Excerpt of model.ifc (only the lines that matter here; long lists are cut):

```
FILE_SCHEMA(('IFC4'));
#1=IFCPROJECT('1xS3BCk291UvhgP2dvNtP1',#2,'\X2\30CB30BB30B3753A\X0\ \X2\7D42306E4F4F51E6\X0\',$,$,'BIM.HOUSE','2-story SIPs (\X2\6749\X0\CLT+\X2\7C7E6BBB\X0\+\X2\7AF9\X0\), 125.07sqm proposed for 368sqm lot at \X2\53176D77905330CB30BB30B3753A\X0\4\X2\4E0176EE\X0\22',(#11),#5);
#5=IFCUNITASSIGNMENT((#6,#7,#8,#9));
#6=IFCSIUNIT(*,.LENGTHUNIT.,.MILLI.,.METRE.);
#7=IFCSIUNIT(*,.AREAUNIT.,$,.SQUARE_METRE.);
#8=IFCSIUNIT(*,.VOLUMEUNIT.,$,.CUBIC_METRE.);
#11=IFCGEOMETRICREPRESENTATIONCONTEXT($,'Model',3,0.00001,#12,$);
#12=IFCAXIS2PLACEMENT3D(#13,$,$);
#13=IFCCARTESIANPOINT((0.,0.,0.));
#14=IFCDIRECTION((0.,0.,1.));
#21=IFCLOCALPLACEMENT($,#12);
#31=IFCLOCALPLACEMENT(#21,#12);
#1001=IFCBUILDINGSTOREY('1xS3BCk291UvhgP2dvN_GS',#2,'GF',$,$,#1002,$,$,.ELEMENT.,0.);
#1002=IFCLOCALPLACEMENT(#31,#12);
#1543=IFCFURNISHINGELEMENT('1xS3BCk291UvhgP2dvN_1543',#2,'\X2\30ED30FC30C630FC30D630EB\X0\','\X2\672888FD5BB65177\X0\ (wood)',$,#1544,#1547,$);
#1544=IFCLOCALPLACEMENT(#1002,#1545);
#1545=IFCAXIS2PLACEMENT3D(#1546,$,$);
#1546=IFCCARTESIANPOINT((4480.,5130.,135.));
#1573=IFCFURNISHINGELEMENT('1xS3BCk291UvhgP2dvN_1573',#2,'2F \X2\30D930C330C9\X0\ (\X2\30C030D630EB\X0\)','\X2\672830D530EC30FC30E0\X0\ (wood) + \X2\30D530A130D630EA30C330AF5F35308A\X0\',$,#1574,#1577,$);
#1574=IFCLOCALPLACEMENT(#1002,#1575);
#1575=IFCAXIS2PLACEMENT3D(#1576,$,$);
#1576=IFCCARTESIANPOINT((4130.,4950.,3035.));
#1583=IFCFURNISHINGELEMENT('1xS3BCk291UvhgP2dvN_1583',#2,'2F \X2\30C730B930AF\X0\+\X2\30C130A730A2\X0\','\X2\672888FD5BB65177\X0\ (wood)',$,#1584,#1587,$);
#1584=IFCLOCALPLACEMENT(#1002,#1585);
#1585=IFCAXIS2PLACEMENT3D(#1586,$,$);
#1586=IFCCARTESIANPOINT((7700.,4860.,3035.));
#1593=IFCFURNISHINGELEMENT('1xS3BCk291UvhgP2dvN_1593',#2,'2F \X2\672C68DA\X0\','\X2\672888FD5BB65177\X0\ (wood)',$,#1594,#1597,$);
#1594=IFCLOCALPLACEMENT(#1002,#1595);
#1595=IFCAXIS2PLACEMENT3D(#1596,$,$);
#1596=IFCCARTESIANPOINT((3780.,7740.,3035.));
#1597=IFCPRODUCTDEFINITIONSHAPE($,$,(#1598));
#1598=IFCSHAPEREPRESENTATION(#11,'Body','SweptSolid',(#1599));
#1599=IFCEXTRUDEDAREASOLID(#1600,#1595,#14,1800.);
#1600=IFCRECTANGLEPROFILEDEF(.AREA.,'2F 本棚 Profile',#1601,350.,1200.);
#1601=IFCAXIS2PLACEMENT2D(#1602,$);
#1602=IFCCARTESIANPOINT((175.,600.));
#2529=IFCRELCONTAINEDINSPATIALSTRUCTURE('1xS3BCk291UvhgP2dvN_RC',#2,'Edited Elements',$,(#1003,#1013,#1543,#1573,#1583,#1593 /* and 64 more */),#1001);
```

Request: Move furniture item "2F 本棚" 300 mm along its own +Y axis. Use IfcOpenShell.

```python
import ifcopenshell
import ifcopenshell.api.geometry
import ifcopenshell.util.placement

model = ifcopenshell.open("model.ifc")

item = model.by_guid("1xS3BCk291UvhgP2dvN_1593")
matrix = ifcopenshell.util.placement.get_local_placement(item.ObjectPlacement)
matrix[:3, 3] += matrix[:3, 1] * 300.0
ifcopenshell.api.geometry.edit_object_placement(model, product=item, matrix=matrix, is_si=False)

print(ifcopenshell.util.placement.get_local_placement(item.ObjectPlacement).round(3) + 0.0)

model.write("model_edited.ifc")
```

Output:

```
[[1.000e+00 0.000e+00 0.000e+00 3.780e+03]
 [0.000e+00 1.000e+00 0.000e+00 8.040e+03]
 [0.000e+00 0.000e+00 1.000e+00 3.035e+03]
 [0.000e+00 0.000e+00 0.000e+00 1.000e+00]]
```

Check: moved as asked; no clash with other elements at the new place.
